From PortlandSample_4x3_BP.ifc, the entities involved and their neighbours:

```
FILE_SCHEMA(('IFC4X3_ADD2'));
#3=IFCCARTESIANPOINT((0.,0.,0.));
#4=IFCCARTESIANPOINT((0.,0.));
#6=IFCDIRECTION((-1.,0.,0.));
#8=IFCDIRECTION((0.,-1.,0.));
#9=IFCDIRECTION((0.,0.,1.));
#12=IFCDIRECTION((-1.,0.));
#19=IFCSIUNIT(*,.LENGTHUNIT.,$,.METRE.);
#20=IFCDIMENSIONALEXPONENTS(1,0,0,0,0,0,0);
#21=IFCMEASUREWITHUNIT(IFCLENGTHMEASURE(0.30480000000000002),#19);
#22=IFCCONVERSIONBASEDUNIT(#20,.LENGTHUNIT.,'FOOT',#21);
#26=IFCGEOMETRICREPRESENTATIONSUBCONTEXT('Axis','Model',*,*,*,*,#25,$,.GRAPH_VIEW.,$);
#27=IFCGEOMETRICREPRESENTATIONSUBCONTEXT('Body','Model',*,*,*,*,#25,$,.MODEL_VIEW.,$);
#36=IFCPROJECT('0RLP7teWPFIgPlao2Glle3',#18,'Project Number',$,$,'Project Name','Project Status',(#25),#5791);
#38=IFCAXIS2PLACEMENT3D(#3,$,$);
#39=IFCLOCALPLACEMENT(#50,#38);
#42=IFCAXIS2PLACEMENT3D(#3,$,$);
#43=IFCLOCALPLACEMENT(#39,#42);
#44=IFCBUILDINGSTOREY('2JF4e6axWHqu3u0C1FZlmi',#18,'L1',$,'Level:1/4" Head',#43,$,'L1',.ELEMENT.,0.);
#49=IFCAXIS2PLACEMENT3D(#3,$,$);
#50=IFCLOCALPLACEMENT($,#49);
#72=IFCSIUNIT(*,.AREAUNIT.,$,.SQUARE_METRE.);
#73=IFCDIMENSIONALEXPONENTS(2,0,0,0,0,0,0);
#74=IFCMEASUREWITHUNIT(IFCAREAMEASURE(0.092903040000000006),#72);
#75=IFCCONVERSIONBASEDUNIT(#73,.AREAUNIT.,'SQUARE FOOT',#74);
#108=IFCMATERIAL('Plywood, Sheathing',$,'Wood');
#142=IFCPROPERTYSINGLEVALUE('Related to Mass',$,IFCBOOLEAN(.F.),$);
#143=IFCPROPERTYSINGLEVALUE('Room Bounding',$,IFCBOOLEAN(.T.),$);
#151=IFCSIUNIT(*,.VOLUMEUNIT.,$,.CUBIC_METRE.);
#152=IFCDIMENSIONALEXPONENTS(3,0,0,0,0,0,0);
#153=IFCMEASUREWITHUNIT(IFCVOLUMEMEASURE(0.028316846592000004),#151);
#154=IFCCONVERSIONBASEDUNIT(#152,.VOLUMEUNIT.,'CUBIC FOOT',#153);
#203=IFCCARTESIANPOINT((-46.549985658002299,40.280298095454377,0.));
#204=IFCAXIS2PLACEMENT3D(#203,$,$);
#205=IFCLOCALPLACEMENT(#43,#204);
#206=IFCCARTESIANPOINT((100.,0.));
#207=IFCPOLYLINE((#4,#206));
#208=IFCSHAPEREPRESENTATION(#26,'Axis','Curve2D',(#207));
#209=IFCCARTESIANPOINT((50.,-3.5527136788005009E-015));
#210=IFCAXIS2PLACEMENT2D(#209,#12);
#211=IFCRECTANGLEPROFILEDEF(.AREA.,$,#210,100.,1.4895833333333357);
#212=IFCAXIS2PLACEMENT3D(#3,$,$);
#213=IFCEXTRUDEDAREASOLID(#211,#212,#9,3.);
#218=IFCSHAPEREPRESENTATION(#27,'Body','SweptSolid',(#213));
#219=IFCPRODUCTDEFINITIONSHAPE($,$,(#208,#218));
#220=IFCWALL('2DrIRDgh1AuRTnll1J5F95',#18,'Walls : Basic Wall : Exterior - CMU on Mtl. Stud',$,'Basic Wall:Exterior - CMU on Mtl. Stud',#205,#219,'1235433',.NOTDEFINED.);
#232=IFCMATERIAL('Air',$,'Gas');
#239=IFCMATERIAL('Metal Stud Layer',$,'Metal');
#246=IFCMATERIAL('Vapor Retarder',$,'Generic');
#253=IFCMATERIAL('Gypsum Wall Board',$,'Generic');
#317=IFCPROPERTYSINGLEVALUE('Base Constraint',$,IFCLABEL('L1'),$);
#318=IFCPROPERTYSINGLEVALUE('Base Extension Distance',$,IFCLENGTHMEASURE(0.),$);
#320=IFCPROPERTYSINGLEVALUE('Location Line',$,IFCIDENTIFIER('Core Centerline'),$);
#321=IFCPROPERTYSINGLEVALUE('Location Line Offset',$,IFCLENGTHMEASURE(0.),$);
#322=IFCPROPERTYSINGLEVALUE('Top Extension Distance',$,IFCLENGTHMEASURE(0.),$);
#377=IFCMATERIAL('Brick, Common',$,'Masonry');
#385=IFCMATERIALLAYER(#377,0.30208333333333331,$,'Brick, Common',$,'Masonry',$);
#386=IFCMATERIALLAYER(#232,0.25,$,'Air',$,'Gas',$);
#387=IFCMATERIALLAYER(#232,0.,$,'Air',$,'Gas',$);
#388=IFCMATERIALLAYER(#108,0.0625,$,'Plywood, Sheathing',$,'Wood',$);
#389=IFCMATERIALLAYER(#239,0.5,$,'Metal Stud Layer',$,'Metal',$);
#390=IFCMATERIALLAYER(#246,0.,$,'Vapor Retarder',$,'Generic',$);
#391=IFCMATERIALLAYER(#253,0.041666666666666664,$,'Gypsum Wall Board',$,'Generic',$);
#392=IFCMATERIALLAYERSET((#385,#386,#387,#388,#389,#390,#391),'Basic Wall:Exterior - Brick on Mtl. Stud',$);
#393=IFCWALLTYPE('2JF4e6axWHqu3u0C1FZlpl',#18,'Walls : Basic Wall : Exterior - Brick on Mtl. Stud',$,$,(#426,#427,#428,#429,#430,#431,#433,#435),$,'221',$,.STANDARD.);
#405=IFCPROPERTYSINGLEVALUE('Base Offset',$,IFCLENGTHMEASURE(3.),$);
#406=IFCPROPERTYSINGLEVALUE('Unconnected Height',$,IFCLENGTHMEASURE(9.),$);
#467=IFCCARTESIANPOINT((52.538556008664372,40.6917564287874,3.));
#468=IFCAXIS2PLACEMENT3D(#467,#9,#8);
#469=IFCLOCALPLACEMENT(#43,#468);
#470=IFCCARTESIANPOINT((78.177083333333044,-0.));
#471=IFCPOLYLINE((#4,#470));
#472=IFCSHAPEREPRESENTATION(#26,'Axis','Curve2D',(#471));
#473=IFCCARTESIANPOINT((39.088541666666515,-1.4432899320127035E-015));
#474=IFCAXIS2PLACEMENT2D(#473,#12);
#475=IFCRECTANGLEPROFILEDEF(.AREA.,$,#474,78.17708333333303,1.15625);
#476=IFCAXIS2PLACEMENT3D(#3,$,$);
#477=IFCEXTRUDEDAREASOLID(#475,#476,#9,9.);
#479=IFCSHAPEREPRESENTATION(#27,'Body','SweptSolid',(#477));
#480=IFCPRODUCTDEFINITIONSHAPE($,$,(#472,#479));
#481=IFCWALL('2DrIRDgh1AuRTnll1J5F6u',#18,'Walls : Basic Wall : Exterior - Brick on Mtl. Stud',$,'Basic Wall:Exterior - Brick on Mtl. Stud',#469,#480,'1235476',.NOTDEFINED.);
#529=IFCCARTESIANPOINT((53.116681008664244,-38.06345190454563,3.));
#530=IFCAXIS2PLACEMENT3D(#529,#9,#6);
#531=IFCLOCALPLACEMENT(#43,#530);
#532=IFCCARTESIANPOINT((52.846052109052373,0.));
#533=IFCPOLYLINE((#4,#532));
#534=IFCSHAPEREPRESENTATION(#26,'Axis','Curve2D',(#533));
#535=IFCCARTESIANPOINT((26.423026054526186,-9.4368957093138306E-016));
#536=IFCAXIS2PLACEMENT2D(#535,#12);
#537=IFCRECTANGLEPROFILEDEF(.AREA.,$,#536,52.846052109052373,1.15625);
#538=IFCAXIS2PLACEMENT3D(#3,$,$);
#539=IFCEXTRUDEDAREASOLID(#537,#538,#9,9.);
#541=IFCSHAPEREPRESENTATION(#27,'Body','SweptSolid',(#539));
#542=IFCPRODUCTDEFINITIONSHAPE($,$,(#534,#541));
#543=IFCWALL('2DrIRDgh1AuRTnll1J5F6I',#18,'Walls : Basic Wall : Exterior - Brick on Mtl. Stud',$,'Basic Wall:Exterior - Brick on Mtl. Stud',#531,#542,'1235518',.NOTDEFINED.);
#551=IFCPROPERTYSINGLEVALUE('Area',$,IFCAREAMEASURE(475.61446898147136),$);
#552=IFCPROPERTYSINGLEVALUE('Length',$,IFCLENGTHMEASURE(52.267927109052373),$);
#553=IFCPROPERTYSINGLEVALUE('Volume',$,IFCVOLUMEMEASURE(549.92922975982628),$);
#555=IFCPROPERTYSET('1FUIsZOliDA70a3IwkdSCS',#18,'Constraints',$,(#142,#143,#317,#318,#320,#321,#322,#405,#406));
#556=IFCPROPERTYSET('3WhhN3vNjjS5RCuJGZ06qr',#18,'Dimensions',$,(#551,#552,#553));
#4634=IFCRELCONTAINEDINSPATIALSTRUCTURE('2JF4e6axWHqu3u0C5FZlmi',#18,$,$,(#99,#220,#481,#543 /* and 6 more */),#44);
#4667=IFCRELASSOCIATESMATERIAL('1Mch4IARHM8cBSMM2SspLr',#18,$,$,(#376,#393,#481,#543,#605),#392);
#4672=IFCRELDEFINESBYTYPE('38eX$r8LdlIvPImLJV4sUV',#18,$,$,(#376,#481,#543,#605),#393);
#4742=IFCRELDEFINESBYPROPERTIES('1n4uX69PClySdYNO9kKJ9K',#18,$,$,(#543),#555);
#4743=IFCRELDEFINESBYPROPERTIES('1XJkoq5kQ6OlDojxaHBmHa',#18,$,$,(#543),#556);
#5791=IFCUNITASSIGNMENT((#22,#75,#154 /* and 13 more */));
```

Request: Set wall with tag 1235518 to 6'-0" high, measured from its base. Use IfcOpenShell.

```python
import ifcopenshell
import ifcopenshell.api.pset
import ifcopenshell.geom
import ifcopenshell.util.element
import ifcopenshell.util.representation
import ifcopenshell.util.shape
import ifcopenshell.util.unit

model = ifcopenshell.open("PortlandSample_4x3_BP.ifc")
unit_scale = ifcopenshell.util.unit.calculate_unit_scale(model)
area_scale = ifcopenshell.util.unit.calculate_unit_scale(model, "AREAUNIT")
volume_scale = ifcopenshell.util.unit.calculate_unit_scale(model, "VOLUMEUNIT")
settings = ifcopenshell.geom.settings()


def volume(element):
    """Net volume in cubic metres, openings subtracted."""
    shape = ifcopenshell.geom.create_shape(settings, element)
    return ifcopenshell.util.shape.get_volume(shape.geometry)


wall = model.by_guid("2DrIRDgh1AuRTnll1J5F6I")
before = volume(wall)

body = ifcopenshell.util.representation.get_representation(wall, "Model", "Body")
solid = body.Items[0]
old_height = solid.Depth
solid.Depth = 72 * 0.0254 / unit_scale
after = volume(wall)
thickness = 0.3524  # wall thickness in metres

# Update the stored height, areas and volumes.
pset = model.by_id(ifcopenshell.util.element.get_pset(wall, "Constraints", should_inherit=False)["id"])
ifcopenshell.api.pset.edit_pset(model, pset=pset, properties={
    "Unconnected Height": model.create_entity("IfcLengthMeasure", solid.Depth),
})
pset = model.by_id(ifcopenshell.util.element.get_pset(wall, "Dimensions", should_inherit=False)["id"])
ifcopenshell.api.pset.edit_pset(model, pset=pset, properties={
    "Area": model.create_entity("IfcAreaMeasure", after / thickness / area_scale),
    "Volume": model.create_entity("IfcVolumeMeasure", after / volume_scale),
})

print(f"height {old_height:g} -> {solid.Depth:g}, volume {before:.3f} -> {after:.3f} m3")

model.write("PortlandSample_4x3_BP_v2.ifc")
```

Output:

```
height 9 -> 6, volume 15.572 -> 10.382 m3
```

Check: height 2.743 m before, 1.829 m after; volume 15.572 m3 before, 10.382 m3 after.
